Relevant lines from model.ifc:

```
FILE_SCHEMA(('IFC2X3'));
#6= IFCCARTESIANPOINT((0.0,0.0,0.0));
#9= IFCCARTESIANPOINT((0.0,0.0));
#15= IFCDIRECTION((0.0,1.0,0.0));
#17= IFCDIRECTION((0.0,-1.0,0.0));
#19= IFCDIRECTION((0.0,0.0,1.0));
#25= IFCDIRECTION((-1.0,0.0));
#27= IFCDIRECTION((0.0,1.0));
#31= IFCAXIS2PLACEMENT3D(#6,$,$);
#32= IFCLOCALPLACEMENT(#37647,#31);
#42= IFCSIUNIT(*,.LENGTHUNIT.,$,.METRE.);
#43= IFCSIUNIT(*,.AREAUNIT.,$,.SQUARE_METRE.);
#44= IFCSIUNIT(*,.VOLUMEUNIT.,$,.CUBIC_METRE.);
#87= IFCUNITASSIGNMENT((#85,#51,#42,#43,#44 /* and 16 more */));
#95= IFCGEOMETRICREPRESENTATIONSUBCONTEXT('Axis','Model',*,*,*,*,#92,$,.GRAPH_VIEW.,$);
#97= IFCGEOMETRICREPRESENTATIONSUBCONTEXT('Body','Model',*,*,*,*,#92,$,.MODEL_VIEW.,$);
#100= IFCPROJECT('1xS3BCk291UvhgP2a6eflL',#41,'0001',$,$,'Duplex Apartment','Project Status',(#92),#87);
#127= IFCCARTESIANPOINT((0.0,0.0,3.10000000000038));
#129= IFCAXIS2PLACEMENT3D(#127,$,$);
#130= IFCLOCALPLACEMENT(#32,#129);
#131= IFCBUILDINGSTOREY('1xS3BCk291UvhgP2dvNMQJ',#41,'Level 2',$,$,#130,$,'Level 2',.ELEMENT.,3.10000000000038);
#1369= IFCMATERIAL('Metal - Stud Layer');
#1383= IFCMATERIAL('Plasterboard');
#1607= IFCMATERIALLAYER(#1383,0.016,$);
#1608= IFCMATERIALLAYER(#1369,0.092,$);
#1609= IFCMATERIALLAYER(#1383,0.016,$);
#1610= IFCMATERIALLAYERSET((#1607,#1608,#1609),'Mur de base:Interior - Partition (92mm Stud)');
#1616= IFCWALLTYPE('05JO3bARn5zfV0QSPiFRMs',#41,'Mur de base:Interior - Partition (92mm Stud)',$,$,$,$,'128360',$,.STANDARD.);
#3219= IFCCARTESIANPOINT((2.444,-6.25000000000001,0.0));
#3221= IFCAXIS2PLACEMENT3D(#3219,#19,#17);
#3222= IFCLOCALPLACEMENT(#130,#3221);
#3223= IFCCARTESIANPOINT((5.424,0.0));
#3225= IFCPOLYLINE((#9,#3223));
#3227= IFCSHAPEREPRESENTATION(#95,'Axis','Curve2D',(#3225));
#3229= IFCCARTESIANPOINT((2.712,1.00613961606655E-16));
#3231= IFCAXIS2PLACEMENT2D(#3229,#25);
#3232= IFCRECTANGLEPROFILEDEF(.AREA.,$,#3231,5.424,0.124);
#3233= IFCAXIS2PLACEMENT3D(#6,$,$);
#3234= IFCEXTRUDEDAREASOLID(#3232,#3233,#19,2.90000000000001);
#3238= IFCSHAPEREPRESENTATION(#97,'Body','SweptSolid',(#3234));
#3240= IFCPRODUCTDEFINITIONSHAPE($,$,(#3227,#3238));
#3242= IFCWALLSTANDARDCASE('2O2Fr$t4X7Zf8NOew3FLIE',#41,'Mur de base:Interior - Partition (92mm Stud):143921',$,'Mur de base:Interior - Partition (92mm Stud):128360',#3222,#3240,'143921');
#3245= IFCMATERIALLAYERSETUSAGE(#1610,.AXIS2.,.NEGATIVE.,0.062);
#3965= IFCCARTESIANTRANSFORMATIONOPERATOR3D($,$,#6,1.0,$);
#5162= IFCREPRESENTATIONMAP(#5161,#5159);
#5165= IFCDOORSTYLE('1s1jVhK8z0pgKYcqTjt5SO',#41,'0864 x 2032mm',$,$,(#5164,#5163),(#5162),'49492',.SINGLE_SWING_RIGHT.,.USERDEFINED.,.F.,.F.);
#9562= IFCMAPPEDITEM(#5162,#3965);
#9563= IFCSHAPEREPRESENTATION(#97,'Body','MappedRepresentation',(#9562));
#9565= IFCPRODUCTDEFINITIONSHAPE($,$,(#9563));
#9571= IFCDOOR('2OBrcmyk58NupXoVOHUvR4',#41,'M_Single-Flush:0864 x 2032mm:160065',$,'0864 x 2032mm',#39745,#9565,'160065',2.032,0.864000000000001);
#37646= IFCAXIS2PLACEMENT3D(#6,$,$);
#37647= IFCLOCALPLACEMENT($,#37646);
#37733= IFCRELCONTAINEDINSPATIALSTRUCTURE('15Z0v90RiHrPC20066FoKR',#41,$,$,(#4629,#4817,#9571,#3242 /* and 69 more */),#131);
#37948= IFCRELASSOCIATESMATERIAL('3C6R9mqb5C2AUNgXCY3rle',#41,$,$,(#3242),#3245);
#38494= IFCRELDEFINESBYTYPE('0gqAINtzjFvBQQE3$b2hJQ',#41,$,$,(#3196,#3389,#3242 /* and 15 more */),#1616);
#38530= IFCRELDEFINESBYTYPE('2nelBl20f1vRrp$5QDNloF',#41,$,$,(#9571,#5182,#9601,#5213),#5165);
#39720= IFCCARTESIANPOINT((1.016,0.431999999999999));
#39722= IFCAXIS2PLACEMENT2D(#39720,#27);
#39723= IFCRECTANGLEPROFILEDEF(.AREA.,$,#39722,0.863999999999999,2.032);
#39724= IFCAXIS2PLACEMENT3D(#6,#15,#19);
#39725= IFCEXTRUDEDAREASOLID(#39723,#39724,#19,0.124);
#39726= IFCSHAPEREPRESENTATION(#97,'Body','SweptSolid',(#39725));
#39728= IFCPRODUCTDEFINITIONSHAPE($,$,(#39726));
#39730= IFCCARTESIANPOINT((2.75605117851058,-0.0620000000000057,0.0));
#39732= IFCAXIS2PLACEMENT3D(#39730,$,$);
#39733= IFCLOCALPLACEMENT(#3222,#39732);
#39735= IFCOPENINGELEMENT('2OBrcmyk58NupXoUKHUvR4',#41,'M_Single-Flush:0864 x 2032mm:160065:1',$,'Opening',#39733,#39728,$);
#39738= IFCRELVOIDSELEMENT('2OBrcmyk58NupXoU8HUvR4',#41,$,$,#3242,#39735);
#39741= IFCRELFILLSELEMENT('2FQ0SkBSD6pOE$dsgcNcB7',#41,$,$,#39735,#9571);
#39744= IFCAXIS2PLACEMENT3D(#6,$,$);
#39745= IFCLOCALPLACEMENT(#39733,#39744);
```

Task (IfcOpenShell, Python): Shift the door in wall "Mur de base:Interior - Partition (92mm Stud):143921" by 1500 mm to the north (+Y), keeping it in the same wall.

```python
import ifcopenshell
import ifcopenshell.api.geometry
import ifcopenshell.util.placement
import ifcopenshell.util.unit

model = ifcopenshell.open("model.ifc")
unit_scale = ifcopenshell.util.unit.calculate_unit_scale(model)

door = model.by_guid("2OBrcmyk58NupXoVOHUvR4")
opening = door.FillsVoids[0].RelatingOpeningElement
wall = opening.VoidsElements[0].RelatingBuildingElement

wall_matrix = ifcopenshell.util.placement.get_local_placement(wall.ObjectPlacement)
shift = wall_matrix[:3, 0] * -1.5 / unit_scale
before = ifcopenshell.util.placement.get_local_placement(door.ObjectPlacement)[:3, 3].copy()

# The door is placed relative to its opening, so it follows when the opening moves.
matrix = ifcopenshell.util.placement.get_local_placement(opening.ObjectPlacement)
matrix[:3, 3] += shift
ifcopenshell.api.geometry.edit_object_placement(
    model, product=opening, matrix=matrix, is_si=False, should_transform_children=True
)

after = ifcopenshell.util.placement.get_local_placement(door.ObjectPlacement)[:3, 3]
print("door moved by", (after - before).round(3) + 0.0)

model.write("model_rev.ifc")
```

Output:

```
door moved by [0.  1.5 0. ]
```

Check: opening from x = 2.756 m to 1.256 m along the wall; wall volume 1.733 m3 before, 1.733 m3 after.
